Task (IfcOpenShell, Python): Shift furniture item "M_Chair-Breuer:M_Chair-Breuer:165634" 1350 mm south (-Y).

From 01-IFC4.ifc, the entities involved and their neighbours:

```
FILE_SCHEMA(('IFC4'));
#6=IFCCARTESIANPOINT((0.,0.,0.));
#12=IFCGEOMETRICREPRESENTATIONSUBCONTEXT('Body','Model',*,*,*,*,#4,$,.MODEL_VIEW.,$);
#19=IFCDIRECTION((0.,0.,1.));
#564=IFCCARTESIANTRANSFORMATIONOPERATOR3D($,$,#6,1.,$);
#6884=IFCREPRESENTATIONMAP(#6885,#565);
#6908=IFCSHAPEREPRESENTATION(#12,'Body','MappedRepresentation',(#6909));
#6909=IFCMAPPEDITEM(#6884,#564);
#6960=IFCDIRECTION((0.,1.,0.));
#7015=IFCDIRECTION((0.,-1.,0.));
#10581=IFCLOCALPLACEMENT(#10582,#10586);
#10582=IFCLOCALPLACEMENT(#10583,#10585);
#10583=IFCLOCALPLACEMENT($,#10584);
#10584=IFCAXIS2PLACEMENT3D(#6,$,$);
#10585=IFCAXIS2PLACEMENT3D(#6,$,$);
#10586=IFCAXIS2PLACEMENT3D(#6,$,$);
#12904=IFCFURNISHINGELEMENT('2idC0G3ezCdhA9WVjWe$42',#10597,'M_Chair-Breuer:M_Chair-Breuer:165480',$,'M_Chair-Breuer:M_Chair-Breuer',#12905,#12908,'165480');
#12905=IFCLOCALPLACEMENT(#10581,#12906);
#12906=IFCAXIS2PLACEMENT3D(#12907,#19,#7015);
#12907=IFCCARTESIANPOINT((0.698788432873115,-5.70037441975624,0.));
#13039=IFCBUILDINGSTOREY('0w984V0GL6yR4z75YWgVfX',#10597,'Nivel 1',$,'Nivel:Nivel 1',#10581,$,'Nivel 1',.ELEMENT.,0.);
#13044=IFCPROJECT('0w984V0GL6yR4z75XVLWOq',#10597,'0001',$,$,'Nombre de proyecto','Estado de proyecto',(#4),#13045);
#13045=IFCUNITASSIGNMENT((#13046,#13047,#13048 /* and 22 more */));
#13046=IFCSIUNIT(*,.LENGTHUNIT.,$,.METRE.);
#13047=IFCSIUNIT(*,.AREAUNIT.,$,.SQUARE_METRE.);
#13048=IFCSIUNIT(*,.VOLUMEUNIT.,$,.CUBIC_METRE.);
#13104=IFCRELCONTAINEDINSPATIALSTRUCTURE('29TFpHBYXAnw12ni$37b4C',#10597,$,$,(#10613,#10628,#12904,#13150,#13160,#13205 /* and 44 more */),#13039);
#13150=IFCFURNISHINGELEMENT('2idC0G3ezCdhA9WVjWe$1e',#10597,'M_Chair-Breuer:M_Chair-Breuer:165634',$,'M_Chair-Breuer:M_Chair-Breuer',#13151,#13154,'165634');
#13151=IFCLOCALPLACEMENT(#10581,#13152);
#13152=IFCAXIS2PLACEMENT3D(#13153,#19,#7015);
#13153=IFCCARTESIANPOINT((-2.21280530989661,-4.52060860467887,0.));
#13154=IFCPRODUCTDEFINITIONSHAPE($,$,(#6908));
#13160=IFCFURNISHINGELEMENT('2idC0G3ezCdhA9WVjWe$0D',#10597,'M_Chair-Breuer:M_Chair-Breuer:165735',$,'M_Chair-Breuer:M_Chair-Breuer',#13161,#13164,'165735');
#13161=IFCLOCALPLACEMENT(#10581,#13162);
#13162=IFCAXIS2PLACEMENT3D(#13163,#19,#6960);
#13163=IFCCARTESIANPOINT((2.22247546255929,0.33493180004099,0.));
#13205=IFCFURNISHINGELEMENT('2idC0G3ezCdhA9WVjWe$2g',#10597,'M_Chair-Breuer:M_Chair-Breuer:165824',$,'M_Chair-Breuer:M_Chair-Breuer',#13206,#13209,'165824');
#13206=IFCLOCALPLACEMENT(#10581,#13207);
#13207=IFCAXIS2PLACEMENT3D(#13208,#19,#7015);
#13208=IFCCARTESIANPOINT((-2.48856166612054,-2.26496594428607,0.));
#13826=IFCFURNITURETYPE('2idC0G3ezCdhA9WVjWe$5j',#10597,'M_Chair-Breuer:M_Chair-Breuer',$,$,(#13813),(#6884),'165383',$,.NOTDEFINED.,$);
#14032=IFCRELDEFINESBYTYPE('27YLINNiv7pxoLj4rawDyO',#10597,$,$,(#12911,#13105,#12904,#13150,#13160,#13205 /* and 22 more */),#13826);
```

```python
import ifcopenshell
import ifcopenshell.api.geometry
import ifcopenshell.util.placement

model = ifcopenshell.open("01-IFC4.ifc")

item = model.by_guid("2idC0G3ezCdhA9WVjWe$1e")
matrix = ifcopenshell.util.placement.get_local_placement(item.ObjectPlacement)
matrix[1, 3] -= 1.35
ifcopenshell.api.geometry.edit_object_placement(model, product=item, matrix=matrix, is_si=False)

print(ifcopenshell.util.placement.get_local_placement(item.ObjectPlacement).round(3) + 0.0)

model.write("01-IFC4_v2.ifc")
```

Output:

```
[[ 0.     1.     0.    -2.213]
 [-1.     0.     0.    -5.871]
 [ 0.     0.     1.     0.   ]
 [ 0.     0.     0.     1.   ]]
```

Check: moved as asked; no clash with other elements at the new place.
